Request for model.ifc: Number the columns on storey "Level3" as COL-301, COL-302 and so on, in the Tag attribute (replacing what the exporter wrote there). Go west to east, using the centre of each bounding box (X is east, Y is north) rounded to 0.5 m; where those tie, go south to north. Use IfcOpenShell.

First a look at what the model holds.

```python
import ifcopenshell
import ifcopenshell.util.element
import ifcopenshell.util.placement

model = ifcopenshell.open("model.ifc")
print(model.schema)
storey = next(s for s in model.by_type("IfcBuildingStorey") if s.Name == "Level3")
columns = [e for e in ifcopenshell.util.element.get_decomposition(storey) if e.is_a("IfcColumn")]
for e in sorted(columns, key=lambda e: e.id()):
    origin = ifcopenshell.util.placement.get_local_placement(e.ObjectPlacement)[:3, 3]
    print(e.id(), e.Tag, e.Name, origin.round(2) + 0.0, sep=" | ")
```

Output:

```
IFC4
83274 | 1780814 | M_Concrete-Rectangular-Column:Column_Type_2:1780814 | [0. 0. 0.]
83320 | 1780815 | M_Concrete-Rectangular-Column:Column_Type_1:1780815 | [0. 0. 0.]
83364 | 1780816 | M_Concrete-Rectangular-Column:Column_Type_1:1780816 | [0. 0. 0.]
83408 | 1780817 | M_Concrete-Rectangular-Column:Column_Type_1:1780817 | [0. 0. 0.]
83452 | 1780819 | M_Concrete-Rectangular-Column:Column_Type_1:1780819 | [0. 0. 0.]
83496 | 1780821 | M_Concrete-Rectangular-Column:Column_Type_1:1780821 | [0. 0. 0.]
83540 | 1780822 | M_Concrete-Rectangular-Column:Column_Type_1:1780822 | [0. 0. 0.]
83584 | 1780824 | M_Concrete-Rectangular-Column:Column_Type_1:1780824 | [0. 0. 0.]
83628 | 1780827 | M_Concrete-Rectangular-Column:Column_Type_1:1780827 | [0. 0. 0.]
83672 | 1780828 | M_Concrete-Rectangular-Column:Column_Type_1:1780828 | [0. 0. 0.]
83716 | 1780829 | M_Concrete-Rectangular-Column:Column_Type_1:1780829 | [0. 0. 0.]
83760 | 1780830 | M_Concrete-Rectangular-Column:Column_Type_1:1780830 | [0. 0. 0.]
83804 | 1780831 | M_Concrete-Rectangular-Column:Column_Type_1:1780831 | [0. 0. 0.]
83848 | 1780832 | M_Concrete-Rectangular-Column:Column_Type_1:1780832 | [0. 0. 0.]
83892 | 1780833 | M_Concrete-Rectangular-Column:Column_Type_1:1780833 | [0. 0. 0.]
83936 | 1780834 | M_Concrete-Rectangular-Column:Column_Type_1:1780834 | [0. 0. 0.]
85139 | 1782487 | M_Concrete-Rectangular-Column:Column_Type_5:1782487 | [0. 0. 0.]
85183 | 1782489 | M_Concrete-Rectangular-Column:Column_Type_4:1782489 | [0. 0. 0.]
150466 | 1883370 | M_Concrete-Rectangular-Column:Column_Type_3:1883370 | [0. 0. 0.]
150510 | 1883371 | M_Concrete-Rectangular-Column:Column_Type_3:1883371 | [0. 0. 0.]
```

```python
import ifcopenshell
import ifcopenshell.geom
import ifcopenshell.util.element
import ifcopenshell.util.shape

model = ifcopenshell.open("model.ifc")
settings = ifcopenshell.geom.settings()
settings.set("use-world-coords", True)


def centre(element):
    shape = ifcopenshell.geom.create_shape(settings, element)
    return ifcopenshell.util.shape.get_bbox_centroid(shape.geometry)


storey = next(s for s in model.by_type("IfcBuildingStorey") if s.Name == "Level3")
columns = [e for e in ifcopenshell.util.element.get_decomposition(storey) if e.is_a("IfcColumn")]

# Insertion points can sit at a corner or the storey origin, so sort by the geometry (in metres).
centres = {e: centre(e) for e in columns}
columns.sort(key=lambda e: (round(centres[e][0] / 0.5), centres[e][1]))

for i, e in enumerate(columns, start=1):
    number = f"COL-3{i:02d}"
    e.Tag = number
    print(e.id(), number)

model.write("model_edited.ifc")
```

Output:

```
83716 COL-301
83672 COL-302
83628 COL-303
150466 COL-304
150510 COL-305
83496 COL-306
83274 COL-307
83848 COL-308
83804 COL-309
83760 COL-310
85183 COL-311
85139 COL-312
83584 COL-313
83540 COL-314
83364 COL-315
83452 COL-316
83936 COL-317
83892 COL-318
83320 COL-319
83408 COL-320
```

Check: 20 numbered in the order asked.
